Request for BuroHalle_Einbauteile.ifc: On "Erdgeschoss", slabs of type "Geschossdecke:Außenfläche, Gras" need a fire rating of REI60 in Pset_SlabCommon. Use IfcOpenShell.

First a look at what the model holds.

```python
import ifcopenshell
import ifcopenshell.util.element

model = ifcopenshell.open("BuroHalle_Einbauteile.ifc")
print(model.schema)
storey = next(s for s in model.by_type("IfcBuildingStorey") if s.Name == "Erdgeschoss")
slabs = [e for e in ifcopenshell.util.element.get_decomposition(storey) if e.is_a("IfcSlab")]
seen = {}
for e in slabs:
    element_type = ifcopenshell.util.element.get_type(e)
    key = (element_type.Name if element_type != e and element_type else None, ifcopenshell.util.element.get_pset(e, "Pset_SlabCommon", "FireRating"))
    seen[key] = seen.get(key, 0) + 1
for (name, value), count in sorted(seen.items(), key=str):
    print(count, "x", name, "|", value)
```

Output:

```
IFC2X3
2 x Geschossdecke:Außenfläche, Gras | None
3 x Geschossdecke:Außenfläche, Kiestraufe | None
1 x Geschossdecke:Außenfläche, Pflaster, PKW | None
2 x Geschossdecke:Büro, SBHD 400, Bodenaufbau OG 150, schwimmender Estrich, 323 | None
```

```python
import ifcopenshell
import ifcopenshell.api.pset
import ifcopenshell.util.element

model = ifcopenshell.open("BuroHalle_Einbauteile.ifc")

storey = next(s for s in model.by_type("IfcBuildingStorey") if s.Name == "Erdgeschoss")
slabs = [e for e in ifcopenshell.util.element.get_decomposition(storey) if e.is_a("IfcSlab")]

count = 0
for e in slabs:
    element_type = ifcopenshell.util.element.get_type(e)
    if element_type in (None, e) or element_type.Name != "Geschossdecke:Außenfläche, Gras":
        continue
    # add_pset returns the element's existing set when there is one.
    pset = ifcopenshell.api.pset.add_pset(model, product=e, name="Pset_SlabCommon")
    ifcopenshell.api.pset.edit_pset(model, pset=pset, properties={"FireRating": "REI60"})
    count += 1

print(count, "slabs updated")

model.write("BuroHalle_Einbauteile_updated.ifc")
```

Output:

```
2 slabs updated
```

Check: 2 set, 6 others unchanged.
